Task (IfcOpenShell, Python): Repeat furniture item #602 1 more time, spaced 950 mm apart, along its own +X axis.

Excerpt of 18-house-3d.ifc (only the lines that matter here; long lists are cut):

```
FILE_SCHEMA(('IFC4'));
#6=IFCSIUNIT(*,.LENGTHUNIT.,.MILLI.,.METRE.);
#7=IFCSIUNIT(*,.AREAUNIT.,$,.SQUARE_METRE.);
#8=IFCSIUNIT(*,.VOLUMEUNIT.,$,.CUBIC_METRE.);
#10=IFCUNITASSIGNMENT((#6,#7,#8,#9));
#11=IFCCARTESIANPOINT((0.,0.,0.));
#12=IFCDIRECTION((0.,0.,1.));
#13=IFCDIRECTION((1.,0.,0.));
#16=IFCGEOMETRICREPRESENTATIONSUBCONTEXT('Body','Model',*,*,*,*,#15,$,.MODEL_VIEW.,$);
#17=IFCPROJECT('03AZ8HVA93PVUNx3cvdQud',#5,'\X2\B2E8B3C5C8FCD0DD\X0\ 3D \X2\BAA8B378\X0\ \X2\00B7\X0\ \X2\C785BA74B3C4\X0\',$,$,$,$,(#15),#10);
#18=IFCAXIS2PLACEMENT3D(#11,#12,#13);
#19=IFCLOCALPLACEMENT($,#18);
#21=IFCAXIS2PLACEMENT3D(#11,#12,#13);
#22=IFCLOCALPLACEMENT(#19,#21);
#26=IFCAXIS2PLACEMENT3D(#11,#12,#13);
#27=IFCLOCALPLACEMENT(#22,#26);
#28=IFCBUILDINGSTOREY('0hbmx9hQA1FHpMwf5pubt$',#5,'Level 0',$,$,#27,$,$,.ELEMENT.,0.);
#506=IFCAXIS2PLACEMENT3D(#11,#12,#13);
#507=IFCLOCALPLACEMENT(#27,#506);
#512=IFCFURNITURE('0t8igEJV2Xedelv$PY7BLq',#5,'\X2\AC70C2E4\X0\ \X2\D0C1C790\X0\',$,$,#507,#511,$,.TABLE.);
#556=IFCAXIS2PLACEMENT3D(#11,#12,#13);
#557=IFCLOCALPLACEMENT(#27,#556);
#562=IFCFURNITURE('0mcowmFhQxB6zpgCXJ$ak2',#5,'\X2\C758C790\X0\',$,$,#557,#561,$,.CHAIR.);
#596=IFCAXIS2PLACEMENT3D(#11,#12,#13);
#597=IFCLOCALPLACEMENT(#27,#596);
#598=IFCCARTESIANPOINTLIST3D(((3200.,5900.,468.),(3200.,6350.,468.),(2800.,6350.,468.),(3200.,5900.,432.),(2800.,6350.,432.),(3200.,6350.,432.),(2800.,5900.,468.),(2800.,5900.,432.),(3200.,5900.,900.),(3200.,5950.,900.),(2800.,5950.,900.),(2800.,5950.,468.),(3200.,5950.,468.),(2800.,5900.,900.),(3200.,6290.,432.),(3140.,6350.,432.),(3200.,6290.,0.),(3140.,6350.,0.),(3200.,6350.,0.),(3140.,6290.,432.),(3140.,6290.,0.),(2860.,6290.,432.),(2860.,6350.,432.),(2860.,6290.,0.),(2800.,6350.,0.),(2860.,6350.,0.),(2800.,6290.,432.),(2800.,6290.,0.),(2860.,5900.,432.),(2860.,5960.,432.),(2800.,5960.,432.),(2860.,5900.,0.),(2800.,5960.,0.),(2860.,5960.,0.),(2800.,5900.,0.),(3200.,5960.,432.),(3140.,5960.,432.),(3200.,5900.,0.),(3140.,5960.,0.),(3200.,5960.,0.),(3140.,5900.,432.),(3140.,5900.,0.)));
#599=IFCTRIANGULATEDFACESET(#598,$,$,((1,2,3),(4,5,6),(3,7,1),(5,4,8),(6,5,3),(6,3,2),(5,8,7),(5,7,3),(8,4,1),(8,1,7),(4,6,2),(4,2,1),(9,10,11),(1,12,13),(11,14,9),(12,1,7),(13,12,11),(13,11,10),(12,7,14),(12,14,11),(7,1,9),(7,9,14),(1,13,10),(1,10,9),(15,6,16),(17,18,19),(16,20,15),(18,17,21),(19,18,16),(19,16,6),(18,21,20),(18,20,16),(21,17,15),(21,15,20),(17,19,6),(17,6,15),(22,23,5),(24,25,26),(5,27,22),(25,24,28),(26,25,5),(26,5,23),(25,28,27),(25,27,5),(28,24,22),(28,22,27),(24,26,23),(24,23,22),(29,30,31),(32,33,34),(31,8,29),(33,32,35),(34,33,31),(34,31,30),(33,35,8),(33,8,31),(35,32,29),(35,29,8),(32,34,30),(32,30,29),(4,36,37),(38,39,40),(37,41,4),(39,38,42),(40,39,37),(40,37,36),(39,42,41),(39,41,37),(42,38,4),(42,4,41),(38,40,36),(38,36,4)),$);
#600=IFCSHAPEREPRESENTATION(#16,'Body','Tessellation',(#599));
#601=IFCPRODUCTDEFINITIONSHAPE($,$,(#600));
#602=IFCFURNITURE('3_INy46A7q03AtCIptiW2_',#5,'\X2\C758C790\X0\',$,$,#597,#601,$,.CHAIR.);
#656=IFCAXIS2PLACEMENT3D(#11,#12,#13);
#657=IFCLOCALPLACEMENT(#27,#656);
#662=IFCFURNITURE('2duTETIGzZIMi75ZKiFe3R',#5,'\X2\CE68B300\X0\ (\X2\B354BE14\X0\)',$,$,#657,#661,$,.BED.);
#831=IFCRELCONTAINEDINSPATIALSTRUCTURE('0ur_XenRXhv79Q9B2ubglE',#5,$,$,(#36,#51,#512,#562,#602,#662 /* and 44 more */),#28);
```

```python
import ifcopenshell
import ifcopenshell.api.geometry
import ifcopenshell.api.root
import ifcopenshell.util.element
import ifcopenshell.util.placement

model = ifcopenshell.open("18-house-3d.ifc")


def reuse_history(source, copy):
    """copy_class also copies each property set's owner history, people and application; keep the originals."""
    for rel in copy.IsDefinedBy:
        if rel.is_a("IfcRelDefinesByProperties") and (history := rel.RelatingPropertyDefinition.OwnerHistory):
            rel.RelatingPropertyDefinition.OwnerHistory = source.OwnerHistory
            ifcopenshell.util.element.remove_deep2(model, history)


source = model.by_guid("3_INy46A7q03AtCIptiW2_")
base = ifcopenshell.util.placement.get_local_placement(source.ObjectPlacement)
step = base[:3, 0] * 950.0

for i in range(1, 2):
    copy = ifcopenshell.api.root.copy_class(model, product=source)
    copy.Representation = ifcopenshell.util.element.copy_deep(
        model, source.Representation, exclude=["IfcGeometricRepresentationContext", "IfcRepresentationMap"]
    )
    reuse_history(source, copy)
    matrix = base.copy()
    matrix[:3, 3] += i * step
    print("added at", matrix[:3, 3].round(3) + 0.0)
    ifcopenshell.api.geometry.edit_object_placement(model, product=copy, matrix=matrix, is_si=False)

model.write("18-house-3d-out.ifc")
```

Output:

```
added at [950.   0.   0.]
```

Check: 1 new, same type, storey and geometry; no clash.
